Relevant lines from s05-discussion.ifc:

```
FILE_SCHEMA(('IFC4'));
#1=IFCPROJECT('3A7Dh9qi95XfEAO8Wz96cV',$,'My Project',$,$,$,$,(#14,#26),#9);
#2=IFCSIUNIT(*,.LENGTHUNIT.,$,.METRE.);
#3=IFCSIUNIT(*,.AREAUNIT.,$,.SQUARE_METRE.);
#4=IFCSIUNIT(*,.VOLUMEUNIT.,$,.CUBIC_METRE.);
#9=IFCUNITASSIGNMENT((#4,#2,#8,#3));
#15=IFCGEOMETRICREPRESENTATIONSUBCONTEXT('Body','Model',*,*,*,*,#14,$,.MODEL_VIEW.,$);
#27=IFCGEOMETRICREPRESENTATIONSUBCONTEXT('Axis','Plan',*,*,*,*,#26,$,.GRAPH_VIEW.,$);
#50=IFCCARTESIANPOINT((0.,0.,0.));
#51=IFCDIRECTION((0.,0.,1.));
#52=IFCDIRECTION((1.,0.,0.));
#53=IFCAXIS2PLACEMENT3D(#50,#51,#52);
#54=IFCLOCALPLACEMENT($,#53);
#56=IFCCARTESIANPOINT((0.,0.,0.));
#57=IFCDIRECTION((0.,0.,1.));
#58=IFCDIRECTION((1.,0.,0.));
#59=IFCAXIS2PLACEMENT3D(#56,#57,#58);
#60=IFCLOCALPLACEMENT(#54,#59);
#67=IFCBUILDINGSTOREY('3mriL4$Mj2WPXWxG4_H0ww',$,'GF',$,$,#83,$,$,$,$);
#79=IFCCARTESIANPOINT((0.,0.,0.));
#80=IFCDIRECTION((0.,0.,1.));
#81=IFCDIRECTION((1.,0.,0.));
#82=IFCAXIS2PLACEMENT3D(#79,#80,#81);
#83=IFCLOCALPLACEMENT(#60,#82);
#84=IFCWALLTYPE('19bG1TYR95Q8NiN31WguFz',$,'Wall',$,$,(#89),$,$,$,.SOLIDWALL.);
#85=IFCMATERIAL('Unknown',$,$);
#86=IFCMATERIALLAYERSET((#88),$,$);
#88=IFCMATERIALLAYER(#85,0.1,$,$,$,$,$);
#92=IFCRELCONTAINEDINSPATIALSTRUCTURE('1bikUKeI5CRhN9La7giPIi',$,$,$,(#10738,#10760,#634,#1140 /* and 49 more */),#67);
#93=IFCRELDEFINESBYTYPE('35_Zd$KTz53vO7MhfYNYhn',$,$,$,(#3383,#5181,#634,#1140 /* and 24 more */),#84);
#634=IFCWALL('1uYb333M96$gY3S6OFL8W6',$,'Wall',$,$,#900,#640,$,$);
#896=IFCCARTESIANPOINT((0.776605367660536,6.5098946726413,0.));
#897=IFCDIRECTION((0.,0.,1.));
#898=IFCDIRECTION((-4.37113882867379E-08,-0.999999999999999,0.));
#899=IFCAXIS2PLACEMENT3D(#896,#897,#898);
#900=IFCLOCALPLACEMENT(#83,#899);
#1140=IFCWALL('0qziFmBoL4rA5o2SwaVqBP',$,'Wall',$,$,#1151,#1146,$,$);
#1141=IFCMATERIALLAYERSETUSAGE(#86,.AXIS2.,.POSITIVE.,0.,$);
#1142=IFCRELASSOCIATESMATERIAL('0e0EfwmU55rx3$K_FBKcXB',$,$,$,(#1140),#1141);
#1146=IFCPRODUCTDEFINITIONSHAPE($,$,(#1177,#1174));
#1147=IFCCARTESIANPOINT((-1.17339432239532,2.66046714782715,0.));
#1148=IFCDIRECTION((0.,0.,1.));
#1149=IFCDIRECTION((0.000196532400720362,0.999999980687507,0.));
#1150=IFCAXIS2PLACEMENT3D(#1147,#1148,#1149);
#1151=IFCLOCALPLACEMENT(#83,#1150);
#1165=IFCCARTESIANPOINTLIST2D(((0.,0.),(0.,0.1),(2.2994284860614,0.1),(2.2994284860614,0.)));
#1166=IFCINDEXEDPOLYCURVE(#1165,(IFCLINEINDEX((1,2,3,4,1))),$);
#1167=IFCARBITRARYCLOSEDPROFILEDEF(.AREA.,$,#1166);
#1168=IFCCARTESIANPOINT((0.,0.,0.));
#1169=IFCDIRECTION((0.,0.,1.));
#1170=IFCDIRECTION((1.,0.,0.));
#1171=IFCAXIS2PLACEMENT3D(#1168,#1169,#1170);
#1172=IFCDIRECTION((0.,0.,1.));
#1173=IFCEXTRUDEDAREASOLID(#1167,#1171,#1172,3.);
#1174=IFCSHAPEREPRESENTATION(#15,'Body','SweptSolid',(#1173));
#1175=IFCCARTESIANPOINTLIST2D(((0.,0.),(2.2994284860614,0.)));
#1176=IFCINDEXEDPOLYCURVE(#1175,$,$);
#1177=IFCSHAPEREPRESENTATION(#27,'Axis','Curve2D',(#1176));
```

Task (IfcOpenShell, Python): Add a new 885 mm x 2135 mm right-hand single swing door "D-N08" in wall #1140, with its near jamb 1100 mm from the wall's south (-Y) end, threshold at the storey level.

```python
import numpy as np
import ifcopenshell
import ifcopenshell.api.feature
import ifcopenshell.api.geometry
import ifcopenshell.api.root
import ifcopenshell.api.spatial
import ifcopenshell.geom
import ifcopenshell.util.element
import ifcopenshell.util.placement
import ifcopenshell.util.representation
import ifcopenshell.util.shape
import ifcopenshell.util.unit

model = ifcopenshell.open("s05-discussion.ifc")
unit_scale = ifcopenshell.util.unit.calculate_unit_scale(model)
settings = ifcopenshell.geom.settings()


def volume(element):
    """Net volume in cubic metres, openings subtracted."""
    shape = ifcopenshell.geom.create_shape(settings, element)
    return ifcopenshell.util.shape.get_volume(shape.geometry)


wall = model.by_guid("0qziFmBoL4rA5o2SwaVqBP")
storey = ifcopenshell.util.element.get_container(wall, ifc_class="IfcBuildingStorey")
context = ifcopenshell.util.representation.get_context(model, "Model", "Body", "MODEL_VIEW")
before = volume(wall)

width, height, from_end, sill = 0.885, 2.135, 1.1, 0.0  # metres

# The wall runs along its own X axis, and the end named is its -X end.
wall_shape = ifcopenshell.geom.create_shape(settings, wall)
x, y, z = ifcopenshell.util.shape.get_vertices(wall_shape.geometry).T
start = x.min() + from_end
face, thickness = float(y.min()), float(y.max() - y.min())
wall_matrix = ifcopenshell.util.placement.get_local_placement(wall.ObjectPlacement)
level = ifcopenshell.util.placement.get_local_placement(storey.ObjectPlacement)[2, 3]


def in_wall(x, y):
    """Placement at x, y metres in the wall's axes, at sill height."""
    matrix = wall_matrix.copy()
    matrix[:, 3] = wall_matrix @ np.array([x / unit_scale, y / unit_scale, 0.0, 1.0])
    matrix[2, 3] = level + sill / unit_scale
    return matrix


# Opening: a box that overshoots both wall faces by 50 mm.
opening = ifcopenshell.api.root.create_entity(model, ifc_class="IfcOpeningElement", predefined_type="OPENING")
box = ifcopenshell.api.geometry.add_wall_representation(
    model, context=context, length=width, height=height, thickness=thickness + 0.1
)
ifcopenshell.api.geometry.assign_representation(model, product=opening, representation=box)
ifcopenshell.api.geometry.edit_object_placement(model, product=opening, matrix=in_wall(start, face - 0.05), is_si=False)
ifcopenshell.api.feature.add_feature(model, feature=opening, element=wall)

door = ifcopenshell.api.root.create_entity(model, ifc_class="IfcDoor", name="D-N08", predefined_type="DOOR")
door.OverallWidth, door.OverallHeight = width / unit_scale, height / unit_scale
door.OperationType = "SINGLE_SWING_RIGHT"
body = ifcopenshell.api.geometry.add_door_representation(
    model,
    context=context,
    overall_width=door.OverallWidth,
    overall_height=door.OverallHeight,
    operation_type="SINGLE_SWING_RIGHT",
    lining_properties={"LiningDepth": thickness / unit_scale, "ThresholdDepth": thickness / unit_scale},
)
ifcopenshell.api.geometry.assign_representation(model, product=door, representation=body)
ifcopenshell.api.spatial.assign_container(model, products=[door], relating_structure=storey)
ifcopenshell.api.feature.add_filling(model, opening=opening, element=door)

# The lining spans the wall, so the door starts at the wall face.
ifcopenshell.api.geometry.edit_object_placement(model, product=door, matrix=in_wall(start, face), is_si=False)

after = volume(wall)

print(f"wall volume {before:.3f} -> {after:.3f} m3")

model.write("s05-discussion_edited.ifc")
```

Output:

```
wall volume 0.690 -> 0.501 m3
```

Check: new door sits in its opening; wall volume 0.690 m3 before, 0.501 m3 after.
